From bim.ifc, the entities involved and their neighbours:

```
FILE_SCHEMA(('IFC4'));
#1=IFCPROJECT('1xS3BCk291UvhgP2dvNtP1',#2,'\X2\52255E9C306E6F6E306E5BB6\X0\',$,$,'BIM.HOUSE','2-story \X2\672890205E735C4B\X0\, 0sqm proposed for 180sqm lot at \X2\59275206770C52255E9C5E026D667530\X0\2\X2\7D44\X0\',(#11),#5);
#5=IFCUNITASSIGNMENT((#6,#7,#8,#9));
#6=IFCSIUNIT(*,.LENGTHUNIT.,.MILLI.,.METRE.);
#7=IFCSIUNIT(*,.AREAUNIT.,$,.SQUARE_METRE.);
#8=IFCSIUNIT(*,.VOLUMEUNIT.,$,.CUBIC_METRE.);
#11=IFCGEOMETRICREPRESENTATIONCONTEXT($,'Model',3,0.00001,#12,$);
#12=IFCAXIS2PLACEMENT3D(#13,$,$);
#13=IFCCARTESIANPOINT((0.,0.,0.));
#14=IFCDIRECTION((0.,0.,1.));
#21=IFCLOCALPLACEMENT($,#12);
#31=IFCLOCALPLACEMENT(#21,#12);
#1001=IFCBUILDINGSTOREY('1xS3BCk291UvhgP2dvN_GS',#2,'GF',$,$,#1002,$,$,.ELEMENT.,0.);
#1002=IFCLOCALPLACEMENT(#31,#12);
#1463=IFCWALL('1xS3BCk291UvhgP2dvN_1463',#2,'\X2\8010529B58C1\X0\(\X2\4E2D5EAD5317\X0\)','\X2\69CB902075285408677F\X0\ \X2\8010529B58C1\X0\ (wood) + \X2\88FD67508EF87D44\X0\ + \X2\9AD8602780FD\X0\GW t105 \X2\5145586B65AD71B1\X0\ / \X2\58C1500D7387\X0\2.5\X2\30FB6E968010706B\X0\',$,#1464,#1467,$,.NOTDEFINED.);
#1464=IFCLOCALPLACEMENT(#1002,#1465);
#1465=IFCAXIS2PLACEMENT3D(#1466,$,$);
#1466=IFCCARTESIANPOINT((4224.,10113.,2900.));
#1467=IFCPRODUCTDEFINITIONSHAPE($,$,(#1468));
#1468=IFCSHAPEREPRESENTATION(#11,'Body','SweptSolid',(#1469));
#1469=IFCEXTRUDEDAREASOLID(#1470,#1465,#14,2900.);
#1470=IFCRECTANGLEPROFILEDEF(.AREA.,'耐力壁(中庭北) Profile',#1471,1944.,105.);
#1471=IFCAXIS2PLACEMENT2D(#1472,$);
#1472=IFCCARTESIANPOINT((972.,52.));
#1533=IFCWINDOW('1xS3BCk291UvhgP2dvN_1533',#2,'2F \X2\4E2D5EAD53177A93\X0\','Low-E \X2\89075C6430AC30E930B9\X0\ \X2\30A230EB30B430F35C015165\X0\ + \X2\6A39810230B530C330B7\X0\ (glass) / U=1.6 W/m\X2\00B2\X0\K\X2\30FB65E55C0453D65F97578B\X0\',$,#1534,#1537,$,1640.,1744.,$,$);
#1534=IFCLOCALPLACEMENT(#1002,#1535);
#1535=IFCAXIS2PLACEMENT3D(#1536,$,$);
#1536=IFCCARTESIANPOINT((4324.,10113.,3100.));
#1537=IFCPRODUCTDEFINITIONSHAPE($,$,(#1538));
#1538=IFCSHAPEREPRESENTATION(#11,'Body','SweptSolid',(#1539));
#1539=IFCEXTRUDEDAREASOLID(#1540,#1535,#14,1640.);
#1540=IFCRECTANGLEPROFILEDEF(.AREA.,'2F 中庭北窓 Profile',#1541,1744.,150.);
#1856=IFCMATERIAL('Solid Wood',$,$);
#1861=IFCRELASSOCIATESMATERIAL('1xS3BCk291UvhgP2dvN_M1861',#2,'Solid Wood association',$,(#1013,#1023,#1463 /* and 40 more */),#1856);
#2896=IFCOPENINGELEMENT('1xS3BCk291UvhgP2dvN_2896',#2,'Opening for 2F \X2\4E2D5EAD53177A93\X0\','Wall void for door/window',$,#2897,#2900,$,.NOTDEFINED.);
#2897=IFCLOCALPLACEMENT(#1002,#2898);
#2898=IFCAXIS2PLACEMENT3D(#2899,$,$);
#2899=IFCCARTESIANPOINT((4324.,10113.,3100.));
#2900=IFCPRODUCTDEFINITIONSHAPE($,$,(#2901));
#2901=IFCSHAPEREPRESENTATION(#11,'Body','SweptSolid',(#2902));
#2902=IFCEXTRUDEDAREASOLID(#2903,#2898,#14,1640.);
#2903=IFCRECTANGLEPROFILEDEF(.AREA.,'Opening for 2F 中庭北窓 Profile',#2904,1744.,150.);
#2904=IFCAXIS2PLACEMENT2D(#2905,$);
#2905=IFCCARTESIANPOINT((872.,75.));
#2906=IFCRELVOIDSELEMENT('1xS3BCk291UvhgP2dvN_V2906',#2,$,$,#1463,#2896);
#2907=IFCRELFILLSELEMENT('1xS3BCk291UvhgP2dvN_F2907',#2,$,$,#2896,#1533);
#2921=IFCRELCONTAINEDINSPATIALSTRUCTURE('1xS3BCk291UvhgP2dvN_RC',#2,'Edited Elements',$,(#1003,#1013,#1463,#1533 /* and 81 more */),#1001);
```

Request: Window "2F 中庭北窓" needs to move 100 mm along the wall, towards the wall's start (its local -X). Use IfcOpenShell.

```python
import ifcopenshell
import ifcopenshell.api.geometry
import ifcopenshell.util.placement
import ifcopenshell.util.unit

model = ifcopenshell.open("bim.ifc")
unit_scale = ifcopenshell.util.unit.calculate_unit_scale(model)

window = model.by_guid("1xS3BCk291UvhgP2dvN_1533")
opening = window.FillsVoids[0].RelatingOpeningElement
wall = opening.VoidsElements[0].RelatingBuildingElement

wall_matrix = ifcopenshell.util.placement.get_local_placement(wall.ObjectPlacement)
shift = wall_matrix[:3, 0] * -0.1 / unit_scale
before = ifcopenshell.util.placement.get_local_placement(window.ObjectPlacement)[:3, 3].copy()

# The window is not placed relative to its opening, so move both.
for product in (opening, window):
    matrix = ifcopenshell.util.placement.get_local_placement(product.ObjectPlacement)
    matrix[:3, 3] += shift
    ifcopenshell.api.geometry.edit_object_placement(model, product=product, matrix=matrix, is_si=False)

after = ifcopenshell.util.placement.get_local_placement(window.ObjectPlacement)[:3, 3]
print("window moved by", (after - before).round(3) + 0.0)

model.write("bim_v2.ifc")
```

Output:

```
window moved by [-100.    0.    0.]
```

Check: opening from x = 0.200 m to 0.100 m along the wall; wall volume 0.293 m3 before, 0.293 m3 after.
